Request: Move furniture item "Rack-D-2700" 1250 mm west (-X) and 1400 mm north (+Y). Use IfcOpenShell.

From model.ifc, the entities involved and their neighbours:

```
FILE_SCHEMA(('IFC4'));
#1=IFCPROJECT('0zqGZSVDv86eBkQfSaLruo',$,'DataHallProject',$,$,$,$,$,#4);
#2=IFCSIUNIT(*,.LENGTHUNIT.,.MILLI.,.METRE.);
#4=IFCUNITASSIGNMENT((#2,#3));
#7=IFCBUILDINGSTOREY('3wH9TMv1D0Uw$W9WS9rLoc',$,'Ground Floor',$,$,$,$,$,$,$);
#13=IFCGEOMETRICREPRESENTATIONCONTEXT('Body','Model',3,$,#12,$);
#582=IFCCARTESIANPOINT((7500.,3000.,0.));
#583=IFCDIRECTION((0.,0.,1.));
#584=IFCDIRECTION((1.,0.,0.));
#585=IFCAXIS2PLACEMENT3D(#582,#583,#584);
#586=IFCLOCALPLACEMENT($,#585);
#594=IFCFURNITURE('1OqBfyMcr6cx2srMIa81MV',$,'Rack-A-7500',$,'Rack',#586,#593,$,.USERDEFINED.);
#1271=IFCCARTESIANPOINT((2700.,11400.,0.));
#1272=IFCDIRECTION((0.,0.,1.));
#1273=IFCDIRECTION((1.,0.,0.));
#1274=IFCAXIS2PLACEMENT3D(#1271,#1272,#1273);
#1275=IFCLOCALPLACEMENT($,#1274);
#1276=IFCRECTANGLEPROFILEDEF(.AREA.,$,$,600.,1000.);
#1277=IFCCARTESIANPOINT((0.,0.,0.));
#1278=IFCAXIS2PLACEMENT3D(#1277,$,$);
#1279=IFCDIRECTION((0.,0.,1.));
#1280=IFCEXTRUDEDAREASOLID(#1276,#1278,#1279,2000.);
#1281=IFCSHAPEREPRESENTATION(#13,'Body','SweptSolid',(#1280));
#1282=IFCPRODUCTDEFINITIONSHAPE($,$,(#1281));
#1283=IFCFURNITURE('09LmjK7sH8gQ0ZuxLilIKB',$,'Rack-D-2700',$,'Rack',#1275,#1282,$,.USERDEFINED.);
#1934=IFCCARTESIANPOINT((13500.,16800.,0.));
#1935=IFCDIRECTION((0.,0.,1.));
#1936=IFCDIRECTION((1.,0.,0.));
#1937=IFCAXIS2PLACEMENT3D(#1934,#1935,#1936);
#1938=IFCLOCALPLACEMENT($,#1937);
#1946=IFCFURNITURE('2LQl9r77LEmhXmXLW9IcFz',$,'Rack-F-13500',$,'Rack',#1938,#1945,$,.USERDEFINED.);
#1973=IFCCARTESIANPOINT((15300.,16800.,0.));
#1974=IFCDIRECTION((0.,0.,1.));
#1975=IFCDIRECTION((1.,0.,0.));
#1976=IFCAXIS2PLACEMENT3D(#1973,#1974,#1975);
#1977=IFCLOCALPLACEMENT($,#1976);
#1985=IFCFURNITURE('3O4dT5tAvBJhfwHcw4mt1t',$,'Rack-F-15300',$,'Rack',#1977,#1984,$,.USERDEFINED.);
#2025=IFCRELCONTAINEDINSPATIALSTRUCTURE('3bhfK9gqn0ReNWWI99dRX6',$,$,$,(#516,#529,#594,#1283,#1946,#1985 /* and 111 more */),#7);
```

```python
import ifcopenshell
import ifcopenshell.api.geometry
import ifcopenshell.util.placement

model = ifcopenshell.open("model.ifc")

item = model.by_id(1283)
matrix = ifcopenshell.util.placement.get_local_placement(item.ObjectPlacement)
matrix[0, 3] -= 1250.0
matrix[1, 3] += 1400.0
ifcopenshell.api.geometry.edit_object_placement(model, product=item, matrix=matrix, is_si=False)

print(ifcopenshell.util.placement.get_local_placement(item.ObjectPlacement).round(3) + 0.0)

model.write("model-out.ifc")
```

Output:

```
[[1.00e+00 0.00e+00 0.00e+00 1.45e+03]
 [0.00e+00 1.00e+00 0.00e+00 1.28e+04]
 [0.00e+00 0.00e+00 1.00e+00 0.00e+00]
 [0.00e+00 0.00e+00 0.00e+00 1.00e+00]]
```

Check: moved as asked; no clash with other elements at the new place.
